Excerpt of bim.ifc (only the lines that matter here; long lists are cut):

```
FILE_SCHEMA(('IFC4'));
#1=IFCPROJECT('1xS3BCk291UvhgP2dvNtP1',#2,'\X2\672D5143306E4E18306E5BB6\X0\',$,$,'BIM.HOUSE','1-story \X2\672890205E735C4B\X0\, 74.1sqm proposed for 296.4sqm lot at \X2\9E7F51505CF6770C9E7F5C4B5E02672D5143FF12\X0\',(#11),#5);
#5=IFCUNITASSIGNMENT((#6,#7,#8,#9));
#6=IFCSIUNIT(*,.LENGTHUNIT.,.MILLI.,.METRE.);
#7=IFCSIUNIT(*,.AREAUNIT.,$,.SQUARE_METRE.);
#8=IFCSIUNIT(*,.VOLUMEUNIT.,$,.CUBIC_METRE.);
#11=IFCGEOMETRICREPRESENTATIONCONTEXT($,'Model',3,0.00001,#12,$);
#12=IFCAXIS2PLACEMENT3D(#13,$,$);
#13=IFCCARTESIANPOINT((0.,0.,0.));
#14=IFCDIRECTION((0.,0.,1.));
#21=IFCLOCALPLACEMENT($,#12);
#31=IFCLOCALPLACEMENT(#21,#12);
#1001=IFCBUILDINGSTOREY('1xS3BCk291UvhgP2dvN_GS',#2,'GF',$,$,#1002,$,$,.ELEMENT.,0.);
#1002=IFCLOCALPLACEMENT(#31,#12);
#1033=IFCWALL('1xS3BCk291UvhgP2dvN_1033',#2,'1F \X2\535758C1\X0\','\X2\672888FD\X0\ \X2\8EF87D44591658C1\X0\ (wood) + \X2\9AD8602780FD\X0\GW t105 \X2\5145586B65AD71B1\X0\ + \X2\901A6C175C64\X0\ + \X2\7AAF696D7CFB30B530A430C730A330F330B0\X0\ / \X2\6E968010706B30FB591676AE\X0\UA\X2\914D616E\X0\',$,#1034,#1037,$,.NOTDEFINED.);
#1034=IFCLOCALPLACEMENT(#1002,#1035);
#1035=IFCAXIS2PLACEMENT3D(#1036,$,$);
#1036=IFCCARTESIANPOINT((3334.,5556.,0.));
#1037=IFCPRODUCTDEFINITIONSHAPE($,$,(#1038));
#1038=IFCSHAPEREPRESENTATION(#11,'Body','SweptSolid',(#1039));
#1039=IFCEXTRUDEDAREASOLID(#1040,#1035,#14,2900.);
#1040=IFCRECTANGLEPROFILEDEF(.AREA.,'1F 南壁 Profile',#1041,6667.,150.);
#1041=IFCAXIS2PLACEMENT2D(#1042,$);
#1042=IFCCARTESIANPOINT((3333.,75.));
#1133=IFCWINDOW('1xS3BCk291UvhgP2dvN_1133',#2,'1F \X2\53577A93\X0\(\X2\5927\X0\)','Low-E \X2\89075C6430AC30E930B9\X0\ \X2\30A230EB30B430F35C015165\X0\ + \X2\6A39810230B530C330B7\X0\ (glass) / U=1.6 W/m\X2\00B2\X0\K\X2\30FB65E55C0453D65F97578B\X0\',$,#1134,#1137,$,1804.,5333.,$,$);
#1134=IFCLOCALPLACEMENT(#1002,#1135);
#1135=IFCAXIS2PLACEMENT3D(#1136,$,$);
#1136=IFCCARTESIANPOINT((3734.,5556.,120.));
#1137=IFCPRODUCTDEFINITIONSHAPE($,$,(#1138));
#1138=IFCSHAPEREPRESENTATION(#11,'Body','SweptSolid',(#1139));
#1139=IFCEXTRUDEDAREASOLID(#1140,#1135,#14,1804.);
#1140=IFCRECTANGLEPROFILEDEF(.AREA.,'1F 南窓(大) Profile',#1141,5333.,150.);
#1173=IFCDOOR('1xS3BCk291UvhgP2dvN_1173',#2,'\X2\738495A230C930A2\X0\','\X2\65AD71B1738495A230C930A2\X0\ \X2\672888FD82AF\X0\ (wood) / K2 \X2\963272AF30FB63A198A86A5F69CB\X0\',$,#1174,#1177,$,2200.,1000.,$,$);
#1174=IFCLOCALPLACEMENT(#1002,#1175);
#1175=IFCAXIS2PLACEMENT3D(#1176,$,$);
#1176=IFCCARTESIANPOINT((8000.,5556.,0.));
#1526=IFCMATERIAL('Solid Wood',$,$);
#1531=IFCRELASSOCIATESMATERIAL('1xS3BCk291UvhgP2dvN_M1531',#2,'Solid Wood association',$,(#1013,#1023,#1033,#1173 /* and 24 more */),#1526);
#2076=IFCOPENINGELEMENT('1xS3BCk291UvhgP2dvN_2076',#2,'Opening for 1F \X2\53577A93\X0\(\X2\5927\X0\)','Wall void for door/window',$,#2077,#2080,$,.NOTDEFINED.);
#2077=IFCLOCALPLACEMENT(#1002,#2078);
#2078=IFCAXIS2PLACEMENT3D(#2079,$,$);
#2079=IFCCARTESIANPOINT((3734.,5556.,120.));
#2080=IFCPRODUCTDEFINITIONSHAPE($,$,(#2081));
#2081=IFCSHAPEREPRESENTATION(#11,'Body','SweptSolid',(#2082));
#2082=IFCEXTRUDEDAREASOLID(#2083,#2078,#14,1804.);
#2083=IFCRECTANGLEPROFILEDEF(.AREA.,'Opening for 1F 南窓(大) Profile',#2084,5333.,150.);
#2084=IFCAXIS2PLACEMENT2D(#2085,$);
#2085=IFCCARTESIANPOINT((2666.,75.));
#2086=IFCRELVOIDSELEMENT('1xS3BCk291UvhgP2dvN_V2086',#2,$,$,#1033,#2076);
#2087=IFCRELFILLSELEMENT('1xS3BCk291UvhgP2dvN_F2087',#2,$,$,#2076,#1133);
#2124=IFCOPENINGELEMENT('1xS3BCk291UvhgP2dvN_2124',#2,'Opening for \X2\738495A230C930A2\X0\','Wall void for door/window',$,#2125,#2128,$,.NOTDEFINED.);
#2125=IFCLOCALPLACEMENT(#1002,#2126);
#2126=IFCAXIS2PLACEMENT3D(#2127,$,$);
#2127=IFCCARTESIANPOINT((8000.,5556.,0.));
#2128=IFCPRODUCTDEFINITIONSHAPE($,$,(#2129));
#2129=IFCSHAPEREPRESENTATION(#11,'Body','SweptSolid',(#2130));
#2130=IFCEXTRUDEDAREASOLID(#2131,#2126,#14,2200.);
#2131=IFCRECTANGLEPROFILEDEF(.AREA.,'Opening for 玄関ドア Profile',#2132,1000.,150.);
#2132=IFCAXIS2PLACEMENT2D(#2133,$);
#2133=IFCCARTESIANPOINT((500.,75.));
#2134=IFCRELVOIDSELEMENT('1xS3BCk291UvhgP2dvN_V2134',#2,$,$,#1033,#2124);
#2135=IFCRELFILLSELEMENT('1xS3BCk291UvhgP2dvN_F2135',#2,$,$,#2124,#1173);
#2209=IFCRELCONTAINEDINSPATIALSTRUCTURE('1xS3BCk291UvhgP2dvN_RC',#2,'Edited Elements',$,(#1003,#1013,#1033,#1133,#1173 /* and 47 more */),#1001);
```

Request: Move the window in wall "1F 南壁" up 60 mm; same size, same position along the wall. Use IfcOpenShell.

```python
import numpy as np
import ifcopenshell
import ifcopenshell.api.geometry
import ifcopenshell.util.placement
import ifcopenshell.util.unit

model = ifcopenshell.open("bim.ifc")
unit_scale = ifcopenshell.util.unit.calculate_unit_scale(model)

window = model.by_guid("1xS3BCk291UvhgP2dvN_1133")
opening = window.FillsVoids[0].RelatingOpeningElement
dz = 60.0

shift = np.array([0.0, 0.0, dz])
# The window is not placed relative to its opening, so move both.
for product in (opening, window):
    matrix = ifcopenshell.util.placement.get_local_placement(product.ObjectPlacement)
    matrix[:3, 3] += shift
    ifcopenshell.api.geometry.edit_object_placement(model, product=product, matrix=matrix, is_si=False)

print(f"moved by {dz * unit_scale:+.3f} m")

model.write("bim_v2.ifc")
```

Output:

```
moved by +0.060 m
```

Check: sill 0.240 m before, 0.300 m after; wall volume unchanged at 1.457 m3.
